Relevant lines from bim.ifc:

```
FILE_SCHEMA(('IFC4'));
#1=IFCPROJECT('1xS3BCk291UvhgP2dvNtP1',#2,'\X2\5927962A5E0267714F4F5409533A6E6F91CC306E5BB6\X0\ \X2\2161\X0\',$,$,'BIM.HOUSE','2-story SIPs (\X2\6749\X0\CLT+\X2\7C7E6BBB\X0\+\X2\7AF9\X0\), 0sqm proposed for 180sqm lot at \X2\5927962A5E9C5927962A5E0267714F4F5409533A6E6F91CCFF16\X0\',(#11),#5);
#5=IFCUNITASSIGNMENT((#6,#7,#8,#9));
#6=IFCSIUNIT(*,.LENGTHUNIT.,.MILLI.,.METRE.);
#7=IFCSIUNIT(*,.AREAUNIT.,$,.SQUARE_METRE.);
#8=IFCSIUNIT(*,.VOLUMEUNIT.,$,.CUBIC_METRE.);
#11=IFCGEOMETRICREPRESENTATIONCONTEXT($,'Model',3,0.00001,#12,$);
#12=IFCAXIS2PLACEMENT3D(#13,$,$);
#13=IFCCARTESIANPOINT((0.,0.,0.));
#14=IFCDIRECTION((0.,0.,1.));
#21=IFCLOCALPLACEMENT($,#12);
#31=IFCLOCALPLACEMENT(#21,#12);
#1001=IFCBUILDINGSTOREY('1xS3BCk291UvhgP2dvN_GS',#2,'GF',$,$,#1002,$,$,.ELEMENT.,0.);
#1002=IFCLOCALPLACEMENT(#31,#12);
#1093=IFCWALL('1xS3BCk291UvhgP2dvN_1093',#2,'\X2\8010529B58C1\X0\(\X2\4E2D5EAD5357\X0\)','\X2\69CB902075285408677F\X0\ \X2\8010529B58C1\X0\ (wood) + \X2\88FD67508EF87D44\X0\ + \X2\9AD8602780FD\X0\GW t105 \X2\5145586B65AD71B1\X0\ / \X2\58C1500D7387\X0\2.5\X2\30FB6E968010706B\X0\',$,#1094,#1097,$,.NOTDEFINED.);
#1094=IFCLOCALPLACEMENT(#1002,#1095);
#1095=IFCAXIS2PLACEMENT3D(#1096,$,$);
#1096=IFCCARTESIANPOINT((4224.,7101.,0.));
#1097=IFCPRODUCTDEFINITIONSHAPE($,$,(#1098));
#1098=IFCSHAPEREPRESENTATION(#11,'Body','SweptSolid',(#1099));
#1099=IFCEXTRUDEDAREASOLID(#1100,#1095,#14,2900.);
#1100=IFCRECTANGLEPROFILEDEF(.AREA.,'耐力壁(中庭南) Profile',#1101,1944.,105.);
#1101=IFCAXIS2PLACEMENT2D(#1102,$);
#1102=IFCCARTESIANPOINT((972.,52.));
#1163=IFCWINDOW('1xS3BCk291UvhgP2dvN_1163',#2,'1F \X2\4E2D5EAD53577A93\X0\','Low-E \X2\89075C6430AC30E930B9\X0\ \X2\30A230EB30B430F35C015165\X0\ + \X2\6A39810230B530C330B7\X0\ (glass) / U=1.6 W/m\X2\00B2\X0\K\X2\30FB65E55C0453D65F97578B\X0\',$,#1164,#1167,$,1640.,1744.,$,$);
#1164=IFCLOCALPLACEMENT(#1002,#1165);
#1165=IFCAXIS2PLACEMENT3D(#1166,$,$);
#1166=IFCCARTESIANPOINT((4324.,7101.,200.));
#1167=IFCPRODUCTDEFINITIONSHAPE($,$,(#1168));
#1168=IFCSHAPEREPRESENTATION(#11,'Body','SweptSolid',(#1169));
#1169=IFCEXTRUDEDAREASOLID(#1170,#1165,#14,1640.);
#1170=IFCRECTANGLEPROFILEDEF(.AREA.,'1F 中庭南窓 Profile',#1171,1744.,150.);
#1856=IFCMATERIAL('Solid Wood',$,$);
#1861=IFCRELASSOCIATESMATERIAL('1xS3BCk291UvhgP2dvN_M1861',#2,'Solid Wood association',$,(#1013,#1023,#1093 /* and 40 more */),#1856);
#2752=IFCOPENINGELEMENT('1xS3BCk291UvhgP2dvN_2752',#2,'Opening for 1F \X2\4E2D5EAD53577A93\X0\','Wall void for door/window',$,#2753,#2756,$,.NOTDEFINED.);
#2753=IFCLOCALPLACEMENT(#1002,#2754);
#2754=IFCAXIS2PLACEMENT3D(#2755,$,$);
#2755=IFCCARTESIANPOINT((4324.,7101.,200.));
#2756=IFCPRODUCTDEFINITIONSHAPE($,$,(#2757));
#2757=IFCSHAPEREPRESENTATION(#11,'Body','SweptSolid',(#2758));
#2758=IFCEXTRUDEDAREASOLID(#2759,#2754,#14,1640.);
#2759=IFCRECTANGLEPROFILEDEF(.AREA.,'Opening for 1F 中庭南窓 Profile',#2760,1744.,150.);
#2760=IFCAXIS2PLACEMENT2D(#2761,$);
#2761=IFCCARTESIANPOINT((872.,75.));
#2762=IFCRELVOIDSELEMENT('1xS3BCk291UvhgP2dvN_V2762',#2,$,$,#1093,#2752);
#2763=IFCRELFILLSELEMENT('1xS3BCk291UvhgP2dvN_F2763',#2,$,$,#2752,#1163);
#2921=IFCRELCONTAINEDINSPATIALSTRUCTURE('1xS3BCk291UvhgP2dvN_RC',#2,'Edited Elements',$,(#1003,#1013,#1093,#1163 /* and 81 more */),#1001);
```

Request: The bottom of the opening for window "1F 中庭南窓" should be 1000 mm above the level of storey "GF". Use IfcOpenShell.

```python
import numpy as np
import ifcopenshell
import ifcopenshell.api.geometry
import ifcopenshell.geom
import ifcopenshell.util.element
import ifcopenshell.util.placement
import ifcopenshell.util.shape
import ifcopenshell.util.unit

model = ifcopenshell.open("bim.ifc")
unit_scale = ifcopenshell.util.unit.calculate_unit_scale(model)

window = model.by_id(1163)
opening = window.FillsVoids[0].RelatingOpeningElement
storey = ifcopenshell.util.element.get_container(window, ifc_class="IfcBuildingStorey")
level = ifcopenshell.util.placement.get_local_placement(storey.ObjectPlacement)[2, 3]

# The opening's origin need not be at the sill, so measure its lowest point.
shape = ifcopenshell.geom.create_shape(ifcopenshell.geom.settings(), opening)
bottom = ifcopenshell.util.shape.get_shape_bottom_elevation(shape, shape.geometry) / unit_scale
dz = level + 1 / unit_scale - bottom

shift = np.array([0.0, 0.0, dz])
# The window is not placed relative to its opening, so move both.
for product in (opening, window):
    matrix = ifcopenshell.util.placement.get_local_placement(product.ObjectPlacement)
    matrix[:3, 3] += shift
    ifcopenshell.api.geometry.edit_object_placement(model, product=product, matrix=matrix, is_si=False)

print(f"moved by {dz * unit_scale:+.3f} m")

model.write("bim_v2.ifc")
```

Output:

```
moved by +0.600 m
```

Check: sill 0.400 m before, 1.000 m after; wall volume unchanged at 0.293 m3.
